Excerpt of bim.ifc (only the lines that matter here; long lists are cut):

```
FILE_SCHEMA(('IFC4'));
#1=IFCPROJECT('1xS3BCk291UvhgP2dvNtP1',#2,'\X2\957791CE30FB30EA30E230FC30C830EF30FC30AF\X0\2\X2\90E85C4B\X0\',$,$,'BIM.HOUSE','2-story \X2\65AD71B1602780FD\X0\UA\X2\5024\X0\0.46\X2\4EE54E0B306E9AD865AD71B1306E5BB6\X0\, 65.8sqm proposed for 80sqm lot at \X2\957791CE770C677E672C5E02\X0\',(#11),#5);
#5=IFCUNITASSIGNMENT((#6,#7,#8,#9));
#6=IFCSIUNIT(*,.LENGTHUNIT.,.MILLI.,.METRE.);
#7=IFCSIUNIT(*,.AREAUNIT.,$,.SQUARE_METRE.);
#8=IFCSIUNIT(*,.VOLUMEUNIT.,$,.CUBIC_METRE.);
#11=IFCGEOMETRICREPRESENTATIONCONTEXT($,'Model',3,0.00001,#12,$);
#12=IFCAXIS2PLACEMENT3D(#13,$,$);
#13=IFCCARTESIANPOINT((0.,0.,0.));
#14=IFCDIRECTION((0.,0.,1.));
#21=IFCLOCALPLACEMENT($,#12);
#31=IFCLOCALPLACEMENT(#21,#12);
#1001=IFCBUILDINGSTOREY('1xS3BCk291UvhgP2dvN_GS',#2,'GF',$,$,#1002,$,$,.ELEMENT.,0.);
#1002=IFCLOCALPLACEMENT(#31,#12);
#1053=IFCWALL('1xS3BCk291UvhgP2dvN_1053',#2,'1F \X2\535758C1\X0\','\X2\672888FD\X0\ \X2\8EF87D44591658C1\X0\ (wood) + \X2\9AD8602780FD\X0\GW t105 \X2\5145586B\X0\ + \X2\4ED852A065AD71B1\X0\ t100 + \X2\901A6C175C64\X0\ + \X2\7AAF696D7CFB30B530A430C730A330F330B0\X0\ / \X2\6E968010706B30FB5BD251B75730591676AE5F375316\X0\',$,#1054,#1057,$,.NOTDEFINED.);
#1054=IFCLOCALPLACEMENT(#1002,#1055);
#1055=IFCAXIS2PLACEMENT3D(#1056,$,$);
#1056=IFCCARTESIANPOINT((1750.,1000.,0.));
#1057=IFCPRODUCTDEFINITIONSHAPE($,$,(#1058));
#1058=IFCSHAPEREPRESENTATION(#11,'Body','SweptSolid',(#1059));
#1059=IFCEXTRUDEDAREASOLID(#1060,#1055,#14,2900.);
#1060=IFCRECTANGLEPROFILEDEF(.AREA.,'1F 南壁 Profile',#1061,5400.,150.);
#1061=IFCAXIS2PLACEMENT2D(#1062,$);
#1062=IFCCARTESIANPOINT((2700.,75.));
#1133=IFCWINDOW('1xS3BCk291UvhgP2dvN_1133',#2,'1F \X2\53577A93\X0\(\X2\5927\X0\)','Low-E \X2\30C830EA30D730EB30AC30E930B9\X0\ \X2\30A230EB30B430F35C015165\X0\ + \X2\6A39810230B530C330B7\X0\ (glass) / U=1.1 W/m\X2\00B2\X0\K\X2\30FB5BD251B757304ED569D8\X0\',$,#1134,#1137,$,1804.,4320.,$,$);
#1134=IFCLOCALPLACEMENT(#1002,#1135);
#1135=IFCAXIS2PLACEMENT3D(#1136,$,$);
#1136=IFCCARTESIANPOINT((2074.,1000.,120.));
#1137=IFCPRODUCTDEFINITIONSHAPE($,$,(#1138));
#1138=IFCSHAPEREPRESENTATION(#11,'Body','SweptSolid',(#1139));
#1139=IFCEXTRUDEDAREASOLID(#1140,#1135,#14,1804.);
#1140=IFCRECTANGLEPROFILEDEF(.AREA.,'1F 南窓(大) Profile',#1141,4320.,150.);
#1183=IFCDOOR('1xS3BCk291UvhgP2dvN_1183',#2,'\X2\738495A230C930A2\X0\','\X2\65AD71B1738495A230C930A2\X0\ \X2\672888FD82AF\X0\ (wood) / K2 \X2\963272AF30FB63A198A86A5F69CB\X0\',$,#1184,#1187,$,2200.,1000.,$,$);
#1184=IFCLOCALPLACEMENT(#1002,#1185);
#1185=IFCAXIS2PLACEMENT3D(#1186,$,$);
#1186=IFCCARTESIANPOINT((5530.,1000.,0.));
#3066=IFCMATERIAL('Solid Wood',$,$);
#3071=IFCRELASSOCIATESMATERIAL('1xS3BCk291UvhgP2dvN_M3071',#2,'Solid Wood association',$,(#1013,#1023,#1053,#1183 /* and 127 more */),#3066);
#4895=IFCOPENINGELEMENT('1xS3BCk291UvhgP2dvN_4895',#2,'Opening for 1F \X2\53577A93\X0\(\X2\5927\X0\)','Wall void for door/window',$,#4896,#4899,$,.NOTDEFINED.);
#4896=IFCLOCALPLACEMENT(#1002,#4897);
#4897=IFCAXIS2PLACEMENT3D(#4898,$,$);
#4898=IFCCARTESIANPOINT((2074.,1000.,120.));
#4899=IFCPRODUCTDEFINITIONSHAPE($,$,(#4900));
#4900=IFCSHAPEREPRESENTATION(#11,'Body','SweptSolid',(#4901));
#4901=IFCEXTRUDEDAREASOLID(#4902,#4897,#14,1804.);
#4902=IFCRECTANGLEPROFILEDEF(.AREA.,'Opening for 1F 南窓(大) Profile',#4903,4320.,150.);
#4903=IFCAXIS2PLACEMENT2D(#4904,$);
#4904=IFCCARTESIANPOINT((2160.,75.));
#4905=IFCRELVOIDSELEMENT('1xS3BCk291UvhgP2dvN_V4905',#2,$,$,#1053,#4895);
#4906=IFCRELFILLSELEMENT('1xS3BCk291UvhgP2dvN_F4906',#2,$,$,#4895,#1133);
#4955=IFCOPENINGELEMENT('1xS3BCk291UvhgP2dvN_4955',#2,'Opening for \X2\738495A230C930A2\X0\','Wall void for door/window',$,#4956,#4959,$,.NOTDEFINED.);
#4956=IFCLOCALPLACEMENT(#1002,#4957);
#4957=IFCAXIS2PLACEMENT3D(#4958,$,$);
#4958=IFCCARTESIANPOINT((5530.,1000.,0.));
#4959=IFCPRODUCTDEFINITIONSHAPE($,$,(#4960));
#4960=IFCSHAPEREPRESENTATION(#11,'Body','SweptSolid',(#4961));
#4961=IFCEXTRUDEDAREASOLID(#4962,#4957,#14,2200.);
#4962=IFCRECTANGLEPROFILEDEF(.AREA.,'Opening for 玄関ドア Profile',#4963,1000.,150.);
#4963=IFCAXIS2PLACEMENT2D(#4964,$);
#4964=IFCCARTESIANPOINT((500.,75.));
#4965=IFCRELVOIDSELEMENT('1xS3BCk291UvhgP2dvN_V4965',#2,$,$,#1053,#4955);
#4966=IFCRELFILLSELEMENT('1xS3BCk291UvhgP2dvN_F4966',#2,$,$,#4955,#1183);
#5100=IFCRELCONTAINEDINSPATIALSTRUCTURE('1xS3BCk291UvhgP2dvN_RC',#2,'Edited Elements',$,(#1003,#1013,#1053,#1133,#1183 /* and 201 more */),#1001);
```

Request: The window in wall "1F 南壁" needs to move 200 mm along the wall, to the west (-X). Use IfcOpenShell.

```python
import ifcopenshell
import ifcopenshell.api.geometry
import ifcopenshell.util.placement
import ifcopenshell.util.unit

model = ifcopenshell.open("bim.ifc")
unit_scale = ifcopenshell.util.unit.calculate_unit_scale(model)

window = model.by_id(1133)
opening = window.FillsVoids[0].RelatingOpeningElement
wall = opening.VoidsElements[0].RelatingBuildingElement

wall_matrix = ifcopenshell.util.placement.get_local_placement(wall.ObjectPlacement)
shift = wall_matrix[:3, 0] * -0.2 / unit_scale
before = ifcopenshell.util.placement.get_local_placement(window.ObjectPlacement)[:3, 3].copy()

# The window is not placed relative to its opening, so move both.
for product in (opening, window):
    matrix = ifcopenshell.util.placement.get_local_placement(product.ObjectPlacement)
    matrix[:3, 3] += shift
    ifcopenshell.api.geometry.edit_object_placement(model, product=product, matrix=matrix, is_si=False)

after = ifcopenshell.util.placement.get_local_placement(window.ObjectPlacement)[:3, 3]
print("window moved by", (after - before).round(3) + 0.0)

model.write("bim_v2.ifc")
```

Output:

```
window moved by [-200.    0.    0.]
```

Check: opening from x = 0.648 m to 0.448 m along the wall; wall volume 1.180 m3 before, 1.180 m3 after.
